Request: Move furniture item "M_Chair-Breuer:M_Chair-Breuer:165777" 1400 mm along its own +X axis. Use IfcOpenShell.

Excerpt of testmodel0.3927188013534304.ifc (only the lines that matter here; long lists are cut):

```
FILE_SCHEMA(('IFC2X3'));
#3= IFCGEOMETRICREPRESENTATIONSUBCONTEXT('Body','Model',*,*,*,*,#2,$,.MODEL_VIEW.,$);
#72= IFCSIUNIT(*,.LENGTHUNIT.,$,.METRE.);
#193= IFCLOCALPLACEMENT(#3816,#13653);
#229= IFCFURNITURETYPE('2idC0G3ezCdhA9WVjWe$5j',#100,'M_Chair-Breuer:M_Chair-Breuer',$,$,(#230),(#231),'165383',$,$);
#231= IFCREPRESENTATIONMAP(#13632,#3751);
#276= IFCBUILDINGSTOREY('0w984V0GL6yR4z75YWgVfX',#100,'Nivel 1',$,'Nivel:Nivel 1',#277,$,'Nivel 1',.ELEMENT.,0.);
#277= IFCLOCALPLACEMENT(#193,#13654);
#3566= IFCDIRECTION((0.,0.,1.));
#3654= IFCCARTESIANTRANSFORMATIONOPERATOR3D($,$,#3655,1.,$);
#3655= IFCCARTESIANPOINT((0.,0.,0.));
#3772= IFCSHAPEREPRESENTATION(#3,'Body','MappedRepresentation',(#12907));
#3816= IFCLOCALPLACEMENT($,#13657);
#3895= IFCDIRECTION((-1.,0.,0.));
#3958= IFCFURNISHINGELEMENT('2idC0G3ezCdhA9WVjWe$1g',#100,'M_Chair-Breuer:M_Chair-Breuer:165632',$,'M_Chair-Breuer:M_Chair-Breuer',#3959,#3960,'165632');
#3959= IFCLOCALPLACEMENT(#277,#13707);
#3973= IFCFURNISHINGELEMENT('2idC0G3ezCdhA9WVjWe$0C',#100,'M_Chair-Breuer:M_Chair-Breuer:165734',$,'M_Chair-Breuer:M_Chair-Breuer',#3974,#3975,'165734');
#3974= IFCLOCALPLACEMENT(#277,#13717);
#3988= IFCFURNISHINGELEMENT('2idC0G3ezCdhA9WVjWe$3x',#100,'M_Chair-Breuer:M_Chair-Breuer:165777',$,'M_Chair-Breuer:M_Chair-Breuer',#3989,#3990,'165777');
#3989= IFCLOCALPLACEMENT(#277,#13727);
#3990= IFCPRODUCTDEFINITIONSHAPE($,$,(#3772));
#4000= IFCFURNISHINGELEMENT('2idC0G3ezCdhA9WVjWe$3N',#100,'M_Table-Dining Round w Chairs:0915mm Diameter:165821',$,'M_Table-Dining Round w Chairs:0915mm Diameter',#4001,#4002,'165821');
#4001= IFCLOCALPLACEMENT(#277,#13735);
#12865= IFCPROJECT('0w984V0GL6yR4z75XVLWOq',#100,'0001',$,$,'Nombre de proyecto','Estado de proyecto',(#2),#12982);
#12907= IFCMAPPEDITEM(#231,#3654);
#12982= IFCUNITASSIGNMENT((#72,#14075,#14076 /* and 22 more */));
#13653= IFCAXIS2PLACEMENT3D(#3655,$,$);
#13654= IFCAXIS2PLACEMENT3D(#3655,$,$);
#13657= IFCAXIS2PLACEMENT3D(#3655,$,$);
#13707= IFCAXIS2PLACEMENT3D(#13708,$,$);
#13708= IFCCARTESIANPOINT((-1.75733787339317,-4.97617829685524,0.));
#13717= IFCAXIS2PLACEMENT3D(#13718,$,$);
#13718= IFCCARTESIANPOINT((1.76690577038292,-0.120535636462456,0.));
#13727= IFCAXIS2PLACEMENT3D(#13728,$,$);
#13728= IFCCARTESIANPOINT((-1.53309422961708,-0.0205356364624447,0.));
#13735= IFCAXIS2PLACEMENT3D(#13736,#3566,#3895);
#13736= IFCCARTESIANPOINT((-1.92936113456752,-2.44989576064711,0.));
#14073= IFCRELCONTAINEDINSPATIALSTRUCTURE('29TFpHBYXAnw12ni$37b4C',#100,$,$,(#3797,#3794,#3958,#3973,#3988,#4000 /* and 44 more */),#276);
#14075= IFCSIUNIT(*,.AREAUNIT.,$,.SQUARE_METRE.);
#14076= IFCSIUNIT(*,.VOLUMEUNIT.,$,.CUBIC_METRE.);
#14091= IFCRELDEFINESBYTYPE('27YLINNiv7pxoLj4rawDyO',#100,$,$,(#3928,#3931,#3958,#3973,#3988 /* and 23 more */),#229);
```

```python
import ifcopenshell
import ifcopenshell.api.geometry
import ifcopenshell.util.placement

model = ifcopenshell.open("testmodel0.3927188013534304.ifc")

item = model.by_guid("2idC0G3ezCdhA9WVjWe$3x")
matrix = ifcopenshell.util.placement.get_local_placement(item.ObjectPlacement)
matrix[:3, 3] += matrix[:3, 0] * 1.4
ifcopenshell.api.geometry.edit_object_placement(model, product=item, matrix=matrix, is_si=False)

print(ifcopenshell.util.placement.get_local_placement(item.ObjectPlacement).round(3) + 0.0)

model.write("testmodel0.3927188013534304-out.ifc")
```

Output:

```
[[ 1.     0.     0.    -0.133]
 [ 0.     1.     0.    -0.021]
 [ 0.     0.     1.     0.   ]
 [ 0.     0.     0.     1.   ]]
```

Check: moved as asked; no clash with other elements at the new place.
